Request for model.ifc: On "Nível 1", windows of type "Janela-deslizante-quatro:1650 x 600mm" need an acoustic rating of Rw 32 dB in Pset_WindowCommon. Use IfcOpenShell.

First a look at what the model holds.

```python
import ifcopenshell
import ifcopenshell.util.element

model = ifcopenshell.open("model.ifc")
print(model.schema)
storey = next(s for s in model.by_type("IfcBuildingStorey") if s.Name == "Nível 1")
windows = [e for e in ifcopenshell.util.element.get_decomposition(storey) if e.is_a("IfcWindow")]
seen = {}
for e in windows:
    element_type = ifcopenshell.util.element.get_type(e)
    key = (element_type.Name if element_type != e and element_type else None, ifcopenshell.util.element.get_pset(e, "Pset_WindowCommon", "AcousticRating"))
    seen[key] = seen.get(key, 0) + 1
for (name, value), count in sorted(seen.items(), key=str):
    print(count, "x", name, "|", value)
```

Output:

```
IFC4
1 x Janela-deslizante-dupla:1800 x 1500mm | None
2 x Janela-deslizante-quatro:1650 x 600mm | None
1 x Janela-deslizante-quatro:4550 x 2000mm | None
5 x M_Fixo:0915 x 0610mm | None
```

```python
import ifcopenshell
import ifcopenshell.api.pset
import ifcopenshell.util.element

model = ifcopenshell.open("model.ifc")

storey = next(s for s in model.by_type("IfcBuildingStorey") if s.Name == "Nível 1")
windows = [e for e in ifcopenshell.util.element.get_decomposition(storey) if e.is_a("IfcWindow")]

count = 0
for e in windows:
    element_type = ifcopenshell.util.element.get_type(e)
    if element_type in (None, e) or element_type.Name != "Janela-deslizante-quatro:1650 x 600mm":
        continue
    # add_pset returns the element's existing set when there is one.
    pset = ifcopenshell.api.pset.add_pset(model, product=e, name="Pset_WindowCommon")
    ifcopenshell.api.pset.edit_pset(model, pset=pset, properties={"AcousticRating": "Rw 32 dB"})
    count += 1

print(count, "windows updated")

model.write("model-out.ifc")
```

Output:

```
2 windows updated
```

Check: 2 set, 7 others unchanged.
